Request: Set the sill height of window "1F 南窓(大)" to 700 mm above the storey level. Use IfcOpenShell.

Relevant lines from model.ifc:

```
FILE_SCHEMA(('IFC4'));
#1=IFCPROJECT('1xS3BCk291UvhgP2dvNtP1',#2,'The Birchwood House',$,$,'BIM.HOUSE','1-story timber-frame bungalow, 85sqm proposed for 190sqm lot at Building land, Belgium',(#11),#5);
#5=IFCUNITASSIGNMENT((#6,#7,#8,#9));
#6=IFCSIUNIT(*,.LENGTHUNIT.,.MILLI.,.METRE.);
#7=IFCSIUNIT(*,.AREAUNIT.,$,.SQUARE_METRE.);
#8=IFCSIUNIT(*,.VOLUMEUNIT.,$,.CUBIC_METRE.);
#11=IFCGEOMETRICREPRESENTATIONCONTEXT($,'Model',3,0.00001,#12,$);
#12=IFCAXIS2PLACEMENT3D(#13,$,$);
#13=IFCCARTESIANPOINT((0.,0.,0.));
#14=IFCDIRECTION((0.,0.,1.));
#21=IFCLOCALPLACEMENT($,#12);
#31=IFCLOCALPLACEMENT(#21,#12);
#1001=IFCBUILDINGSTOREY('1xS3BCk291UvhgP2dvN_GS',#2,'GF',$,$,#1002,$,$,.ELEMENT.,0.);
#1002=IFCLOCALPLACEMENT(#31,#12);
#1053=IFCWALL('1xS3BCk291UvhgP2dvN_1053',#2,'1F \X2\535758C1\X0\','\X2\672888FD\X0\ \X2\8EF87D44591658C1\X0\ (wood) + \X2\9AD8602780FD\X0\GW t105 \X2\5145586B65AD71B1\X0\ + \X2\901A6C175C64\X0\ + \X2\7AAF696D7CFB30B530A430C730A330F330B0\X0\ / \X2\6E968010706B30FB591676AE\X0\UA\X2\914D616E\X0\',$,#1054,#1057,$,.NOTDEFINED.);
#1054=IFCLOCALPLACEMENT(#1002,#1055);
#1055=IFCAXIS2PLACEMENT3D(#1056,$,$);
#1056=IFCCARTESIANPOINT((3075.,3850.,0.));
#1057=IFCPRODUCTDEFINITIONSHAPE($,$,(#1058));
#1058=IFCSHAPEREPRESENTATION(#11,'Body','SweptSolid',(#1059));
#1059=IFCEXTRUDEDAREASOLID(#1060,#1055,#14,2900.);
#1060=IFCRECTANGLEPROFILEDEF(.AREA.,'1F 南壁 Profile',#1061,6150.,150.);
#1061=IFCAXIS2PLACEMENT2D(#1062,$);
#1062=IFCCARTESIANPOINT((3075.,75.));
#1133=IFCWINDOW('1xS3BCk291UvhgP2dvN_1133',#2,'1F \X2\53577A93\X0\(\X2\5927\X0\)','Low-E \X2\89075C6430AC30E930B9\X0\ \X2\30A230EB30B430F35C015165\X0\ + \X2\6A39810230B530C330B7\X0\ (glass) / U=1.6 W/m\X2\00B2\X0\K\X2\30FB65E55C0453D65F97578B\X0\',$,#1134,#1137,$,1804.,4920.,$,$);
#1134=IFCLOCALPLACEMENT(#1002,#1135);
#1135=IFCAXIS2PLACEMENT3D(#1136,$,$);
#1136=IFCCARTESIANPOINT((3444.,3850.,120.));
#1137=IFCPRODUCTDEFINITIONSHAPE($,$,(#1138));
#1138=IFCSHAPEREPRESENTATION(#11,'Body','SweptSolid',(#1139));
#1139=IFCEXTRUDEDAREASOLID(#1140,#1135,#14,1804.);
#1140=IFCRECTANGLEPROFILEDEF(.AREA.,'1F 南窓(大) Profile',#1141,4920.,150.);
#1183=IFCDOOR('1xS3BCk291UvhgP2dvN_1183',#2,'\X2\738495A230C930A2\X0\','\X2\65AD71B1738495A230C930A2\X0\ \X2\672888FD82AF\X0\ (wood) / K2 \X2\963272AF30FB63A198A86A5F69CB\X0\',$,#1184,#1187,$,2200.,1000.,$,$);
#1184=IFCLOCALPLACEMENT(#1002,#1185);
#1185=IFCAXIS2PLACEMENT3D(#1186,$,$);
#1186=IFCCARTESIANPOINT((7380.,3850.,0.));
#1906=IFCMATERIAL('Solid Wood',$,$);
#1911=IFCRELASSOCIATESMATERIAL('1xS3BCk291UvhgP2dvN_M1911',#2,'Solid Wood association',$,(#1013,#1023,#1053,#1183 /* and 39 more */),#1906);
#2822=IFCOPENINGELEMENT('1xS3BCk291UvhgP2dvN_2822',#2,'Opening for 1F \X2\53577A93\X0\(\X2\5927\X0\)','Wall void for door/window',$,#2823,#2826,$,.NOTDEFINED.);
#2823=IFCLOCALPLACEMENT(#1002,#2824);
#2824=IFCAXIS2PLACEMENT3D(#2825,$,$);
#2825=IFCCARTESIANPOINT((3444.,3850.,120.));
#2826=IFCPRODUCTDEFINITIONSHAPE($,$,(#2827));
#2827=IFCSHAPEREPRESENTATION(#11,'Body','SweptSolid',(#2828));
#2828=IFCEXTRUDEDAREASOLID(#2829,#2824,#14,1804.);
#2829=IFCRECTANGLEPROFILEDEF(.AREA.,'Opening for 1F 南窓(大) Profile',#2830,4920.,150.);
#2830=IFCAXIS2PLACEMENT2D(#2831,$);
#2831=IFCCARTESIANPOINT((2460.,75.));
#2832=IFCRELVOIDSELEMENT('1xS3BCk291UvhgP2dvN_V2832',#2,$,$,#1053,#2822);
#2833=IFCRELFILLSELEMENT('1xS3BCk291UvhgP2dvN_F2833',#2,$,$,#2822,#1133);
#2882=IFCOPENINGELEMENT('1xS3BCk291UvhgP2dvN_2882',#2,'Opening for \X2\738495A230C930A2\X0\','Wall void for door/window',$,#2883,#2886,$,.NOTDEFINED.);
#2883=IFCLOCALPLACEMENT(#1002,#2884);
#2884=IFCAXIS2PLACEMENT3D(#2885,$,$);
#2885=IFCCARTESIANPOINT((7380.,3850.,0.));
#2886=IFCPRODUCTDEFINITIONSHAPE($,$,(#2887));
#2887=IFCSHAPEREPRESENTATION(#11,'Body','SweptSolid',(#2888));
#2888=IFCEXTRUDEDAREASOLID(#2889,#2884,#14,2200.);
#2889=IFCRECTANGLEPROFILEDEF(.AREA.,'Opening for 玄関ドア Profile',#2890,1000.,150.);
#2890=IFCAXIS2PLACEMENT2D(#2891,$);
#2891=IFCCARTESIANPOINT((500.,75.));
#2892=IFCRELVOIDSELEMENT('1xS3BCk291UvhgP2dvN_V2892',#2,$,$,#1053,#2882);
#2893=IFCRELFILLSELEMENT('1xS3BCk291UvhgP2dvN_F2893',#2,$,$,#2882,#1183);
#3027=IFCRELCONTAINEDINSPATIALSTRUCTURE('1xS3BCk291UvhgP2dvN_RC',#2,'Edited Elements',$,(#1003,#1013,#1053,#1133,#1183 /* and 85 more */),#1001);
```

```python
import numpy as np
import ifcopenshell
import ifcopenshell.api.geometry
import ifcopenshell.geom
import ifcopenshell.util.element
import ifcopenshell.util.placement
import ifcopenshell.util.shape
import ifcopenshell.util.unit

model = ifcopenshell.open("model.ifc")
unit_scale = ifcopenshell.util.unit.calculate_unit_scale(model)

window = model.by_id(1133)
opening = window.FillsVoids[0].RelatingOpeningElement
storey = ifcopenshell.util.element.get_container(window, ifc_class="IfcBuildingStorey")
level = ifcopenshell.util.placement.get_local_placement(storey.ObjectPlacement)[2, 3]

# The opening's origin need not be at the sill, so measure its lowest point.
shape = ifcopenshell.geom.create_shape(ifcopenshell.geom.settings(), opening)
bottom = ifcopenshell.util.shape.get_shape_bottom_elevation(shape, shape.geometry) / unit_scale
dz = level + 0.7 / unit_scale - bottom

shift = np.array([0.0, 0.0, dz])
# The window is not placed relative to its opening, so move both.
for product in (opening, window):
    matrix = ifcopenshell.util.placement.get_local_placement(product.ObjectPlacement)
    matrix[:3, 3] += shift
    ifcopenshell.api.geometry.edit_object_placement(model, product=product, matrix=matrix, is_si=False)

print(f"moved by {dz * unit_scale:+.3f} m")

model.write("model_updated.ifc")
```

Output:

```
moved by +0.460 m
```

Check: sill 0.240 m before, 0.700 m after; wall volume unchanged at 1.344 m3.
